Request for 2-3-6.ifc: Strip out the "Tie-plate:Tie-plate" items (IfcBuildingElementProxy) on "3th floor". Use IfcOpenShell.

First a look at what the model holds.

```python
import ifcopenshell
import ifcopenshell.util.element

model = ifcopenshell.open("2-3-6.ifc")
print(model.schema)
storey = next(s for s in model.by_type("IfcBuildingStorey") if s.Name == "3th floor")
proxies = [e for e in ifcopenshell.util.element.get_decomposition(storey) if e.is_a("IfcBuildingElementProxy")]
seen = {}
for e in proxies:
    element_type = ifcopenshell.util.element.get_type(e)
    name = element_type.Name if element_type not in (None, e) else None
    seen[name] = seen.get(name, 0) + 1
for name, count in sorted(seen.items(), key=str):
    print(count, "x", name)
```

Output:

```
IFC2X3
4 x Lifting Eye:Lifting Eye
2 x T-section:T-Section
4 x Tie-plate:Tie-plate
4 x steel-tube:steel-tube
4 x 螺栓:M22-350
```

```python
import ifcopenshell
import ifcopenshell.api.root
import ifcopenshell.util.element

model = ifcopenshell.open("2-3-6.ifc")

storey = next(s for s in model.by_type("IfcBuildingStorey") if s.Name == "3th floor")
proxies = [e for e in ifcopenshell.util.element.get_decomposition(storey) if e.is_a("IfcBuildingElementProxy")]
targets = [e for e in proxies if (t := ifcopenshell.util.element.get_type(e)) not in (None, e) and t.Name == "Tie-plate:Tie-plate"]

for e in targets:
    ifcopenshell.api.root.remove_product(model, product=e)
print(len(targets), "removed")

model.write("2-3-6_rev.ifc")
```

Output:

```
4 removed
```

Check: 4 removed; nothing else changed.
